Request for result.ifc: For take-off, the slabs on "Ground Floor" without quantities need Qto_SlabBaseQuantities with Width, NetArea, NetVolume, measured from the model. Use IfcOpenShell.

First a look at what the model holds.

```python
import ifcopenshell
import ifcopenshell.util.element
import ifcopenshell.util.unit

model = ifcopenshell.open("result.ifc")
print(model.schema)
for unit_type in ("LENGTHUNIT", "AREAUNIT", "VOLUMEUNIT"):
    print(unit_type, ifcopenshell.util.unit.calculate_unit_scale(model, unit_type))
storey = next(s for s in model.by_type("IfcBuildingStorey") if s.Name == "Ground Floor")
slabs = [e for e in ifcopenshell.util.element.get_decomposition(storey) if e.is_a("IfcSlab")]
for e in sorted(slabs, key=lambda e: e.id()):
    print(e.id(), e.is_a(), e.Name, list(ifcopenshell.util.element.get_psets(e, qtos_only=True)), sep=" | ")
```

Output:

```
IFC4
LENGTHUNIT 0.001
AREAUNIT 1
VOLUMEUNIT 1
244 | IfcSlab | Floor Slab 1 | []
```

```python
import ifcopenshell
import ifcopenshell.api.pset
import ifcopenshell.geom
import ifcopenshell.util.element
import ifcopenshell.util.shape
import ifcopenshell.util.unit

model = ifcopenshell.open("result.ifc")
unit_scale = ifcopenshell.util.unit.calculate_unit_scale(model)
area_scale = ifcopenshell.util.unit.calculate_unit_scale(model, "AREAUNIT")
volume_scale = ifcopenshell.util.unit.calculate_unit_scale(model, "VOLUMEUNIT")
settings = ifcopenshell.geom.settings()

storey = next(s for s in model.by_type("IfcBuildingStorey") if s.Name == "Ground Floor")
slabs = [e for e in ifcopenshell.util.element.get_decomposition(storey) if e.is_a("IfcSlab")]

for e in sorted(slabs, key=lambda e: e.id()):
    if ifcopenshell.util.element.get_psets(e, qtos_only=True, should_inherit=False):
        continue
    # Geometry comes back in metres, in the element's own axes.
    shape = ifcopenshell.geom.create_shape(settings, e)
    values = {
        "Width": ifcopenshell.util.shape.get_z(shape.geometry) / unit_scale,
        "NetArea": ifcopenshell.util.shape.get_footprint_area(shape.geometry) / area_scale,
        "NetVolume": ifcopenshell.util.shape.get_volume(shape.geometry) / volume_scale,
    }
    qto = ifcopenshell.api.pset.add_qto(model, product=e, name="Qto_SlabBaseQuantities")
    ifcopenshell.api.pset.edit_qto(model, qto=qto, properties=values)
    print(e.id(), {k: round(v, 3) for k, v in values.items()})

model.write("result-out.ifc")
```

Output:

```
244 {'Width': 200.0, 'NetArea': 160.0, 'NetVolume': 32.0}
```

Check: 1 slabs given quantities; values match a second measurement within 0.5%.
